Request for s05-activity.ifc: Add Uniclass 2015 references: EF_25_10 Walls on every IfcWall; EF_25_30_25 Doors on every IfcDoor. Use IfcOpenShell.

First a look at what the model holds.

```python
import ifcopenshell

model = ifcopenshell.open("s05-activity.ifc")
print(model.schema)
print("classifications:", [c.Name for c in model.by_type("IfcClassification")])
for ifc_class in ("IfcDoor", "IfcRoof", "IfcStair", "IfcWall", "IfcWindow"):
    print(ifc_class, len(model.by_type(ifc_class)))
```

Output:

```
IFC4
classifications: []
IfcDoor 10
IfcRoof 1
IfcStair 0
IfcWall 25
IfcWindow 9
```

```python
import ifcopenshell
import ifcopenshell.api.classification

model = ifcopenshell.open("s05-activity.ifc")

system = ifcopenshell.api.classification.add_classification(model, classification="Uniclass 2015")

codes = {
    "IfcWall": ("EF_25_10", "Walls"),
    "IfcDoor": ("EF_25_30_25", "Doors"),
}
for ifc_class, (code, name) in codes.items():
    products = model.by_type(ifc_class)
    ifcopenshell.api.classification.add_reference(
        model, products=products, classification=system, identification=code, name=name
    )
    print(code, len(products))

model.write("s05-activity_edited.ifc")
```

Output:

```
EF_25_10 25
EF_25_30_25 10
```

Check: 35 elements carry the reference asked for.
